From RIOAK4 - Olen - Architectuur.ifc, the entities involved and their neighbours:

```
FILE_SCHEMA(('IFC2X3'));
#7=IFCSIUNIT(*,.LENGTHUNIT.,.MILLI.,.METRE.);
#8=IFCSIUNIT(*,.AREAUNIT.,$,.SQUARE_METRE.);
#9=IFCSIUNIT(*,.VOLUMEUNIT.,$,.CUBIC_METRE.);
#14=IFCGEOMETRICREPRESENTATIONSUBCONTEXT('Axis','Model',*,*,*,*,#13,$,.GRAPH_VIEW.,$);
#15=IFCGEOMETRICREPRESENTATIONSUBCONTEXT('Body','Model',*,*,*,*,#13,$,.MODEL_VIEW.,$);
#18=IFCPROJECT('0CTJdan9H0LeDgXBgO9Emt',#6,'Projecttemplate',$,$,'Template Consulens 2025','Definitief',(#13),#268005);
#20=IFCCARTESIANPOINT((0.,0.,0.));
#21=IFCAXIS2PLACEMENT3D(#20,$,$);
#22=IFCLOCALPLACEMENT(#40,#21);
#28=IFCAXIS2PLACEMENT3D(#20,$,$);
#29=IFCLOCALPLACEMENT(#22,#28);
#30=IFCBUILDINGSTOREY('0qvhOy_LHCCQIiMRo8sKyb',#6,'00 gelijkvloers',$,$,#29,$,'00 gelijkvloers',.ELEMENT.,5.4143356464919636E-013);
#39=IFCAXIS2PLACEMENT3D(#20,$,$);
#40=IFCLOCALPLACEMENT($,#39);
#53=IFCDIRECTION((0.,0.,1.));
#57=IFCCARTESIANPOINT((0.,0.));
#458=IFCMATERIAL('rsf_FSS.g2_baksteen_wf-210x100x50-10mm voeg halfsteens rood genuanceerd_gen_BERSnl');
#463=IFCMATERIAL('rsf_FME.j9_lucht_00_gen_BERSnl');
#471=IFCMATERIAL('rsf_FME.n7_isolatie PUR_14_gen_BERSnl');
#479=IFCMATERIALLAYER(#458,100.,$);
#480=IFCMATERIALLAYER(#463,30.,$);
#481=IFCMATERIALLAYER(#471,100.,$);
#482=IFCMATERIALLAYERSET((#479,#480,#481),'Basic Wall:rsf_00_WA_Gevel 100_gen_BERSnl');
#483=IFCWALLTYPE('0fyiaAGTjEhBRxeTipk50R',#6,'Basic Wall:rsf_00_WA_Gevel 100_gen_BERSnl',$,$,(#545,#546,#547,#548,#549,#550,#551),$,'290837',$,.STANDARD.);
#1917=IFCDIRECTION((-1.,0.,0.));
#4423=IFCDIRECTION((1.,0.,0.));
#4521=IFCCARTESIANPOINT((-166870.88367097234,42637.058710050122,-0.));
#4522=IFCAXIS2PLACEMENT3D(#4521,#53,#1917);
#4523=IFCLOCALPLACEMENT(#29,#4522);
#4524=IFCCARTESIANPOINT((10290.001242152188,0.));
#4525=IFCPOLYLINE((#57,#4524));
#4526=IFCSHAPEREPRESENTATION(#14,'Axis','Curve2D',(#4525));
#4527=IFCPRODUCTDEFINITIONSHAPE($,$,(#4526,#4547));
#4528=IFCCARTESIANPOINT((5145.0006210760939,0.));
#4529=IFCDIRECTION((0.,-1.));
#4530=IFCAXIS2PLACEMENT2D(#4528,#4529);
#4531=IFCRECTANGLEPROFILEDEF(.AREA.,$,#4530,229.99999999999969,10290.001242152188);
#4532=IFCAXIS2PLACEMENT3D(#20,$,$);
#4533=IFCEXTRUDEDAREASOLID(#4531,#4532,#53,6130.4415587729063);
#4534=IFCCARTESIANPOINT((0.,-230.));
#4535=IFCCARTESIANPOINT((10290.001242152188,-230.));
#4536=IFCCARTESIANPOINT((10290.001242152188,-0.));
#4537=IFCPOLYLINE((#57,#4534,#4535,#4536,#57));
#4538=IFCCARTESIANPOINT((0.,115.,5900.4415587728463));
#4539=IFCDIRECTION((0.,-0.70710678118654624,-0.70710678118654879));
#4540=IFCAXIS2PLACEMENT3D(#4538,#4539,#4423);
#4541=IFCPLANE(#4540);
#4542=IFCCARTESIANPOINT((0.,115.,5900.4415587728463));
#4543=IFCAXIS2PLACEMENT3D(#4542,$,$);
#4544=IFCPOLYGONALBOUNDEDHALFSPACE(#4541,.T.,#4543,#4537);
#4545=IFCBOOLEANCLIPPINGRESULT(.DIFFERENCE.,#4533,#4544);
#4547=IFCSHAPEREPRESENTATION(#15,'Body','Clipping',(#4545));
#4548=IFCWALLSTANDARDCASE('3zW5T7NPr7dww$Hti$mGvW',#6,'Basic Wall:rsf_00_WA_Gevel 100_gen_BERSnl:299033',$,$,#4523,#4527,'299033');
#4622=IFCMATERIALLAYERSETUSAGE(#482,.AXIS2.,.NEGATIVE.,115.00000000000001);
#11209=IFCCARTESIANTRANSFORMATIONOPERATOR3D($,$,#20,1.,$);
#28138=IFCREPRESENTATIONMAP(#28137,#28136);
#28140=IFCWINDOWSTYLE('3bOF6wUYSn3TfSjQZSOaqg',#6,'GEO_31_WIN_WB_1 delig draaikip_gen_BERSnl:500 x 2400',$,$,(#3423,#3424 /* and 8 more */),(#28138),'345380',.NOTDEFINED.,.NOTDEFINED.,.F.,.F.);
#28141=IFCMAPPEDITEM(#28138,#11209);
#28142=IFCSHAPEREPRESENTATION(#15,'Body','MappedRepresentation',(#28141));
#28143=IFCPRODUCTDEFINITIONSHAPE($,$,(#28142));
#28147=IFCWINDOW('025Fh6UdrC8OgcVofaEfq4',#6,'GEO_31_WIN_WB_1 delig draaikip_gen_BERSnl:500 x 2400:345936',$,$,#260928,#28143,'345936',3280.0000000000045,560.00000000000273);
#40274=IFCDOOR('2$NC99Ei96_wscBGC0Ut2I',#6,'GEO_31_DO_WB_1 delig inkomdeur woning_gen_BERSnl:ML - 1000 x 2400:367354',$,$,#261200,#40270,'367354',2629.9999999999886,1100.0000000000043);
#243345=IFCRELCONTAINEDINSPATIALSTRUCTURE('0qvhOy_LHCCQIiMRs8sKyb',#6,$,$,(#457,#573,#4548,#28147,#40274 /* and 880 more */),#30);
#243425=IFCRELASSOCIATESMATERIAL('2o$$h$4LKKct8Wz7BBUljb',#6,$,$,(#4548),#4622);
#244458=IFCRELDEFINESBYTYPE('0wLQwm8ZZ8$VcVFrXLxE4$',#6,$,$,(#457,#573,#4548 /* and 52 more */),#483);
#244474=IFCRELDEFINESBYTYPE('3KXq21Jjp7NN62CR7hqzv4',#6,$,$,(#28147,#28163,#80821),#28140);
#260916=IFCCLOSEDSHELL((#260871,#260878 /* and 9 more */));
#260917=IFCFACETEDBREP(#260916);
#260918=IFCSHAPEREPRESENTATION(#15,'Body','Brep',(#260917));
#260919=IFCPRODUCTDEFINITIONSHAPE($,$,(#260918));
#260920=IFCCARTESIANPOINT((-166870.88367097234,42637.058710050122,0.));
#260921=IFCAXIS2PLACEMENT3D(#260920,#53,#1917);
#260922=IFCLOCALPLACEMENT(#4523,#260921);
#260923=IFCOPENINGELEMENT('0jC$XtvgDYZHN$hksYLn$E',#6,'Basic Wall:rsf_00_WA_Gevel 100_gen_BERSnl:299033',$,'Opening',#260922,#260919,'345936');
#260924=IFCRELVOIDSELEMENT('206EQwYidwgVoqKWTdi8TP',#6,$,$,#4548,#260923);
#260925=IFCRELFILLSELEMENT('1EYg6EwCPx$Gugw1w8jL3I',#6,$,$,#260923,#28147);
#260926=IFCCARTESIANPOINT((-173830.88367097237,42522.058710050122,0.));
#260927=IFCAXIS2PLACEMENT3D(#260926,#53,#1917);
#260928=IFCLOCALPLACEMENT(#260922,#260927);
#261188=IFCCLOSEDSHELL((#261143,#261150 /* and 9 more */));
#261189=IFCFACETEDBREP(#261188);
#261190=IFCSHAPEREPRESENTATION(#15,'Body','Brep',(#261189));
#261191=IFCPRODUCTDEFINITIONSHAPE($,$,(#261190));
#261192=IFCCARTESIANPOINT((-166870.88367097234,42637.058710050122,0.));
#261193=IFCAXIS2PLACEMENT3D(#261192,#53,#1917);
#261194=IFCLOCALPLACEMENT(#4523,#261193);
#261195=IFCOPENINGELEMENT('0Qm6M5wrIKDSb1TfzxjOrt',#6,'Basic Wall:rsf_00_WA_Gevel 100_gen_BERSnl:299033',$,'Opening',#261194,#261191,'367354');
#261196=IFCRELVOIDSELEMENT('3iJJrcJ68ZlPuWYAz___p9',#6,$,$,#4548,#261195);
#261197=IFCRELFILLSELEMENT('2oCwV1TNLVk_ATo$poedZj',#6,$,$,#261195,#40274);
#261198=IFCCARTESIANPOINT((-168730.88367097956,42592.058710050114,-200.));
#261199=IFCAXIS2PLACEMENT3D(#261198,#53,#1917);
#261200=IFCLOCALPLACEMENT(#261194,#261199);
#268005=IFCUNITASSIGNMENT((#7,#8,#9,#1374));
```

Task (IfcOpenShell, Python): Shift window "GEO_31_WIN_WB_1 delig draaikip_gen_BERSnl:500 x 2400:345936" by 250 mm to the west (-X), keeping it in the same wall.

```python
import ifcopenshell
import ifcopenshell.api.geometry
import ifcopenshell.util.placement

model = ifcopenshell.open("RIOAK4 - Olen - Architectuur.ifc")

window = model.by_guid("025Fh6UdrC8OgcVofaEfq4")
opening = window.FillsVoids[0].RelatingOpeningElement
wall = opening.VoidsElements[0].RelatingBuildingElement

wall_matrix = ifcopenshell.util.placement.get_local_placement(wall.ObjectPlacement)
shift = wall_matrix[:3, 0] * 250.0
before = ifcopenshell.util.placement.get_local_placement(window.ObjectPlacement)[:3, 3].copy()

# The window is placed relative to its opening, so it follows when the opening moves.
matrix = ifcopenshell.util.placement.get_local_placement(opening.ObjectPlacement)
matrix[:3, 3] += shift
ifcopenshell.api.geometry.edit_object_placement(
    model, product=opening, matrix=matrix, is_si=False, should_transform_children=True
)

after = ifcopenshell.util.placement.get_local_placement(window.ObjectPlacement)[:3, 3]
print("window moved by", (after - before).round(3) + 0.0)

model.write("RIOAK4 - Olen - Architectuur_v2.ifc")
```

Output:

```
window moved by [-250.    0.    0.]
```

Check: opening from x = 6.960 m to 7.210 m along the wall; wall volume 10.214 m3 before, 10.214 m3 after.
